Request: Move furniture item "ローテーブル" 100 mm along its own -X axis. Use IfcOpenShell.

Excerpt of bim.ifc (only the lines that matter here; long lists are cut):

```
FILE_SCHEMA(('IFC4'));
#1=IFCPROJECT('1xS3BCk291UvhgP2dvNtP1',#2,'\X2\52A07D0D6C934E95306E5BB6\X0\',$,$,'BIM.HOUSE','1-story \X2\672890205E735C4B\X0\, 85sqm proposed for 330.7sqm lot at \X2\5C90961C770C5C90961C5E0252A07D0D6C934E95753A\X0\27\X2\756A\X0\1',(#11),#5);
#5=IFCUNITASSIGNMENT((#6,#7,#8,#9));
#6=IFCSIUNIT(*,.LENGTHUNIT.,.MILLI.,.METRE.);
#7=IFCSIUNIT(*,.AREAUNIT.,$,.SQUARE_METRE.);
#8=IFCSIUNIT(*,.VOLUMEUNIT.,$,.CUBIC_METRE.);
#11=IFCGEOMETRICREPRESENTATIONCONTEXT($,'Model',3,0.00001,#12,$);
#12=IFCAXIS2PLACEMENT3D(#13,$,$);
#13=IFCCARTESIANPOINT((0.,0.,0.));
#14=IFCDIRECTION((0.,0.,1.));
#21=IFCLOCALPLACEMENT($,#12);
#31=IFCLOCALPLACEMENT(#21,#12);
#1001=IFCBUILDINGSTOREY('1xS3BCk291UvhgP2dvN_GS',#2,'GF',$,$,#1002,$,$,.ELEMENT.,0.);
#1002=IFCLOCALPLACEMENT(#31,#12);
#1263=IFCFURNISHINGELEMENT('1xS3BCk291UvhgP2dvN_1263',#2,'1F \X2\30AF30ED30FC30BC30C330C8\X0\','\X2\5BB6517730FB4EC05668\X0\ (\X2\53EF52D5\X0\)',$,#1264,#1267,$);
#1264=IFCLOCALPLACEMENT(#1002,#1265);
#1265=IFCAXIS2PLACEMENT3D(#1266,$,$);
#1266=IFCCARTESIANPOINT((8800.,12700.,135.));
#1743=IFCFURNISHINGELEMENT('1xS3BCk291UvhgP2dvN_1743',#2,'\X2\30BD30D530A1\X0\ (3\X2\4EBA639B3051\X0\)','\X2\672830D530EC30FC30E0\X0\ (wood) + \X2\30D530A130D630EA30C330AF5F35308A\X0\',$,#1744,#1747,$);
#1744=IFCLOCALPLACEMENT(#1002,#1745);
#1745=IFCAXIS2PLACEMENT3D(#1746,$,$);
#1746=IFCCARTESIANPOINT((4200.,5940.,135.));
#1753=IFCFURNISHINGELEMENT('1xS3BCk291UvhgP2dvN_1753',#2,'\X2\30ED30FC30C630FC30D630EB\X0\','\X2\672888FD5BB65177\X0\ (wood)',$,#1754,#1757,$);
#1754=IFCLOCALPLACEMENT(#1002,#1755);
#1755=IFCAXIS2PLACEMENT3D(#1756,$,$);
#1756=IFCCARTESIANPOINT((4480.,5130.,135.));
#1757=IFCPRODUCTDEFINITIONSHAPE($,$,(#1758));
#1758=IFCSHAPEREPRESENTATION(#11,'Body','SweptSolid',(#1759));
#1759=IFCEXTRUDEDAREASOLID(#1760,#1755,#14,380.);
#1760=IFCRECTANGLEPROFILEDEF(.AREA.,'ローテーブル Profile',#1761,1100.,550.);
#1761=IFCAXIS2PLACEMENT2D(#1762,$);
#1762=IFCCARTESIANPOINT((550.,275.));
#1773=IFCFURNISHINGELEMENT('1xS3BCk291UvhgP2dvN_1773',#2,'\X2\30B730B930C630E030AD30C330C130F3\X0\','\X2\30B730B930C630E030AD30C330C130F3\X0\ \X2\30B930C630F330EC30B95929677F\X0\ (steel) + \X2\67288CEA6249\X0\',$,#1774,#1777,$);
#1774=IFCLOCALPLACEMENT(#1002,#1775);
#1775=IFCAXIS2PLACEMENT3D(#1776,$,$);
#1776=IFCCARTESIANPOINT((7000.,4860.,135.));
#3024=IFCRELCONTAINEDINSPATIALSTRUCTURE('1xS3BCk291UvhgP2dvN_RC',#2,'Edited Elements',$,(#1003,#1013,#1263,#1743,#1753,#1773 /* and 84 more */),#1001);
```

```python
import ifcopenshell
import ifcopenshell.api.geometry
import ifcopenshell.util.placement
import ifcopenshell.util.unit

model = ifcopenshell.open("bim.ifc")
unit_scale = ifcopenshell.util.unit.calculate_unit_scale(model)

item = model.by_guid("1xS3BCk291UvhgP2dvN_1753")
matrix = ifcopenshell.util.placement.get_local_placement(item.ObjectPlacement)
matrix[:3, 3] -= matrix[:3, 0] * 0.1 / unit_scale
ifcopenshell.api.geometry.edit_object_placement(model, product=item, matrix=matrix, is_si=False)

print(ifcopenshell.util.placement.get_local_placement(item.ObjectPlacement).round(3) + 0.0)

model.write("bim_updated.ifc")
```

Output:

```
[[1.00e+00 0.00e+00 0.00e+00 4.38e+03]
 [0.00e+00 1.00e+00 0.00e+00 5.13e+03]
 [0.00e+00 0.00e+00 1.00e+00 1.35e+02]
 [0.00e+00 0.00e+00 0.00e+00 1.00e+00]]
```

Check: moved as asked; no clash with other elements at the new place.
